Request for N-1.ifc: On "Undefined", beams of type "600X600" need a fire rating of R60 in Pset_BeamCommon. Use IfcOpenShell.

First a look at what the model holds.

```python
import ifcopenshell
import ifcopenshell.util.element

model = ifcopenshell.open("N-1.ifc")
print(model.schema)
storey = next(s for s in model.by_type("IfcBuildingStorey") if s.Name == "Undefined")
beams = [e for e in ifcopenshell.util.element.get_decomposition(storey) if e.is_a("IfcBeam")]
seen = {}
for e in beams:
    element_type = ifcopenshell.util.element.get_type(e)
    key = (element_type.Name if element_type != e and element_type else None, ifcopenshell.util.element.get_pset(e, "Pset_BeamCommon", "FireRating"))
    seen[key] = seen.get(key, 0) + 1
for (name, value), count in sorted(seen.items(), key=str):
    print(count, "x", name, "|", value)
```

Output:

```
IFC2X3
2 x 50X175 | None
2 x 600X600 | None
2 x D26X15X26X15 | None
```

```python
import ifcopenshell
import ifcopenshell.api.pset
import ifcopenshell.util.element

model = ifcopenshell.open("N-1.ifc")

storey = next(s for s in model.by_type("IfcBuildingStorey") if s.Name == "Undefined")
beams = [e for e in ifcopenshell.util.element.get_decomposition(storey) if e.is_a("IfcBeam")]

count = 0
for e in beams:
    element_type = ifcopenshell.util.element.get_type(e)
    if element_type in (None, e) or element_type.Name != "600X600":
        continue
    found = ifcopenshell.util.element.get_pset(e, "Pset_BeamCommon", should_inherit=False)
    if found:
        pset = model.by_id(found["id"])
        if len(ifcopenshell.util.element.get_elements_by_pset(pset)) > 1:
            pset = ifcopenshell.api.pset.unshare_pset(model, products=[e], pset=pset)[0]
    else:
        pset = ifcopenshell.api.pset.add_pset(model, product=e, name="Pset_BeamCommon")
    ifcopenshell.api.pset.edit_pset(model, pset=pset, properties={"FireRating": "R60"})
    count += 1

print(count, "beams updated")

model.write("N-1_edited.ifc")
```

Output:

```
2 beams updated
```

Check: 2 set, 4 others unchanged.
